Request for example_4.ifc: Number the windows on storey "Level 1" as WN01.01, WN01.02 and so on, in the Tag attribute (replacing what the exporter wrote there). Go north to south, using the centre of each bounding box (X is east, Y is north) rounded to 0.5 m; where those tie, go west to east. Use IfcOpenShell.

First a look at what the model holds.

```python
import ifcopenshell
import ifcopenshell.util.element
import ifcopenshell.util.placement

model = ifcopenshell.open("example_4.ifc")
print(model.schema)
storey = next(s for s in model.by_type("IfcBuildingStorey") if s.Name == "Level 1")
windows = [e for e in ifcopenshell.util.element.get_decomposition(storey) if e.is_a("IfcWindow")]
for e in sorted(windows, key=lambda e: e.id()):
    origin = ifcopenshell.util.placement.get_local_placement(e.ObjectPlacement)[:3, 3]
    print(e.id(), e.Tag, e.Name, origin.round(2) + 0.0, sep=" | ")
```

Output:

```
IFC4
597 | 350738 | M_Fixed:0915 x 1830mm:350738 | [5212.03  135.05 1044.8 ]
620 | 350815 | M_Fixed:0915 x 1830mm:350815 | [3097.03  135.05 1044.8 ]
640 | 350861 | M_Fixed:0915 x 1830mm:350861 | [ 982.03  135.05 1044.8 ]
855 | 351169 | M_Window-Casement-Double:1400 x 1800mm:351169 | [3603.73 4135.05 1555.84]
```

```python
import ifcopenshell
import ifcopenshell.geom
import ifcopenshell.util.element
import ifcopenshell.util.shape

model = ifcopenshell.open("example_4.ifc")
settings = ifcopenshell.geom.settings()
settings.set("use-world-coords", True)


def centre(element):
    shape = ifcopenshell.geom.create_shape(settings, element)
    return ifcopenshell.util.shape.get_bbox_centroid(shape.geometry)


storey = next(s for s in model.by_type("IfcBuildingStorey") if s.Name == "Level 1")
windows = [e for e in ifcopenshell.util.element.get_decomposition(storey) if e.is_a("IfcWindow")]

# Insertion points can sit at a corner or the storey origin, so sort by the geometry (in metres).
centres = {e: centre(e) for e in windows}
windows.sort(key=lambda e: (-round(centres[e][1] / 0.5), centres[e][0]))

for i, e in enumerate(windows, start=1):
    number = f"WN01.{i:02d}"
    e.Tag = number
    print(e.id(), number)

model.write("example_4_rev.ifc")
```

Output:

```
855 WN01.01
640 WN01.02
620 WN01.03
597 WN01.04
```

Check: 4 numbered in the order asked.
